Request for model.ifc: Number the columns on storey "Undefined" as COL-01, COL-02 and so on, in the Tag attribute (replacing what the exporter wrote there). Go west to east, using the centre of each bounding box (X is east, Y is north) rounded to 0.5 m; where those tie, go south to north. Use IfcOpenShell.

First a look at what the model holds.

```python
import ifcopenshell
import ifcopenshell.util.element
import ifcopenshell.util.placement

model = ifcopenshell.open("model.ifc")
print(model.schema)
storey = next(s for s in model.by_type("IfcBuildingStorey") if s.Name == "Undefined")
columns = [e for e in ifcopenshell.util.element.get_decomposition(storey) if e.is_a("IfcColumn")]
for e in sorted(columns, key=lambda e: e.id()):
    origin = ifcopenshell.util.placement.get_local_placement(e.ObjectPlacement)[:3, 3]
    print(e.id(), e.Tag, e.Name, origin.round(2) + 0.0, sep=" | ")
```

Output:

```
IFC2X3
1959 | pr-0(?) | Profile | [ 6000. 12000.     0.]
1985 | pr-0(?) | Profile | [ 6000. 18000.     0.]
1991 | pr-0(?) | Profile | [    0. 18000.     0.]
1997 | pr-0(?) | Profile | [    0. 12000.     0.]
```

```python
import ifcopenshell
import ifcopenshell.geom
import ifcopenshell.util.element
import ifcopenshell.util.shape

model = ifcopenshell.open("model.ifc")
settings = ifcopenshell.geom.settings()
settings.set("use-world-coords", True)


def centre(element):
    shape = ifcopenshell.geom.create_shape(settings, element)
    return ifcopenshell.util.shape.get_bbox_centroid(shape.geometry)


storey = next(s for s in model.by_type("IfcBuildingStorey") if s.Name == "Undefined")
columns = [e for e in ifcopenshell.util.element.get_decomposition(storey) if e.is_a("IfcColumn")]

# Insertion points can sit at a corner or the storey origin, so sort by the geometry (in metres).
centres = {e: centre(e) for e in columns}
columns.sort(key=lambda e: (round(centres[e][0] / 0.5), centres[e][1]))

for i, e in enumerate(columns, start=1):
    number = f"COL-{i:02d}"
    e.Tag = number
    print(e.id(), number)

model.write("model_rev.ifc")
```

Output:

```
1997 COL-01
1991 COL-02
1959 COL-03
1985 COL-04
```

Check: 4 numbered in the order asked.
